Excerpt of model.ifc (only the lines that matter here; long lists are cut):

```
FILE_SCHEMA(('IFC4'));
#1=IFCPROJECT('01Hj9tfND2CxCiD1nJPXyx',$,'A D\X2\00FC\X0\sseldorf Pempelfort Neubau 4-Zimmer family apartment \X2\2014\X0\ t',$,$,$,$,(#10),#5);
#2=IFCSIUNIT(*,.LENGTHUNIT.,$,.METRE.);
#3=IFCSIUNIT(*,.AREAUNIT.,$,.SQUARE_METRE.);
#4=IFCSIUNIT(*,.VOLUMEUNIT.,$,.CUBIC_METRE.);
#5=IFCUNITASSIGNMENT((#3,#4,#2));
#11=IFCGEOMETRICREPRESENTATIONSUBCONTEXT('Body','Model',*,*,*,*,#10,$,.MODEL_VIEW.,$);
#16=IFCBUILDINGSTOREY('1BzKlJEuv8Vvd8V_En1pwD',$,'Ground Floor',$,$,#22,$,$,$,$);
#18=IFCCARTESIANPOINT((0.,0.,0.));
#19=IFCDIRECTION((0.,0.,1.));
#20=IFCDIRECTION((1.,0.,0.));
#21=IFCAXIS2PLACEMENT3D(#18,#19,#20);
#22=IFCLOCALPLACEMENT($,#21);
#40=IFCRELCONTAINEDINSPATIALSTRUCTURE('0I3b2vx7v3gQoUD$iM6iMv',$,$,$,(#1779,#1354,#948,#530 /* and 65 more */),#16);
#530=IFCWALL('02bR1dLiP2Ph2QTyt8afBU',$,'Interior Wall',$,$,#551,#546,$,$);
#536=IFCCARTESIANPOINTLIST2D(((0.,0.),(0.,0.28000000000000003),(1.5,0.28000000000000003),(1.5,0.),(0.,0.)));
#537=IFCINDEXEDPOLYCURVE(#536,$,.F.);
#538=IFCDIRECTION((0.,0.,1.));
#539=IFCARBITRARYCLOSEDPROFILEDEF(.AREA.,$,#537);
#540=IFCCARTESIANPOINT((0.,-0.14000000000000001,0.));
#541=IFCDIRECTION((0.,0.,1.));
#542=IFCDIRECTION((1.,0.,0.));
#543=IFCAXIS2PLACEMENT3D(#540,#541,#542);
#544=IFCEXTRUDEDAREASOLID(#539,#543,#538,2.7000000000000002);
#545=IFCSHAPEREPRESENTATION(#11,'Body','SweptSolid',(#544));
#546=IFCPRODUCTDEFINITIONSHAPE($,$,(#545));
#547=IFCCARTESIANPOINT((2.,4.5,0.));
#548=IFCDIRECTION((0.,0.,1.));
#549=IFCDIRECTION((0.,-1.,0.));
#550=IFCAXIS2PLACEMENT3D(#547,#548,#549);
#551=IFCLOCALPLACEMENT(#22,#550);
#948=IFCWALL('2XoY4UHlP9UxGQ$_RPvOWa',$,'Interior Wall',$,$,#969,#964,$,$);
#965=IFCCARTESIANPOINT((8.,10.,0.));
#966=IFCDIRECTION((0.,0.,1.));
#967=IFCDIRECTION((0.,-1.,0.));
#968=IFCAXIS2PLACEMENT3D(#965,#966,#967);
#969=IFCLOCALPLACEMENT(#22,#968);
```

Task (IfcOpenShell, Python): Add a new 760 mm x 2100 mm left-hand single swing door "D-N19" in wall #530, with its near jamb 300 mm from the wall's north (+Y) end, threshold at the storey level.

```python
import numpy as np
import ifcopenshell
import ifcopenshell.api.feature
import ifcopenshell.api.geometry
import ifcopenshell.api.root
import ifcopenshell.api.spatial
import ifcopenshell.geom
import ifcopenshell.util.element
import ifcopenshell.util.placement
import ifcopenshell.util.representation
import ifcopenshell.util.shape
import ifcopenshell.util.unit

model = ifcopenshell.open("model.ifc")
unit_scale = ifcopenshell.util.unit.calculate_unit_scale(model)
settings = ifcopenshell.geom.settings()


def volume(element):
    """Net volume in cubic metres, openings subtracted."""
    shape = ifcopenshell.geom.create_shape(settings, element)
    return ifcopenshell.util.shape.get_volume(shape.geometry)


wall = model.by_guid("02bR1dLiP2Ph2QTyt8afBU")
storey = ifcopenshell.util.element.get_container(wall, ifc_class="IfcBuildingStorey")
context = ifcopenshell.util.representation.get_context(model, "Model", "Body", "MODEL_VIEW")
before = volume(wall)

width, height, from_end, sill = 0.76, 2.1, 0.3, 0.0  # metres

# The wall runs along its own X axis, and the end named is its -X end.
wall_shape = ifcopenshell.geom.create_shape(settings, wall)
x, y, z = ifcopenshell.util.shape.get_vertices(wall_shape.geometry).T
start = x.min() + from_end
face, thickness = float(y.min()), float(y.max() - y.min())
wall_matrix = ifcopenshell.util.placement.get_local_placement(wall.ObjectPlacement)
level = ifcopenshell.util.placement.get_local_placement(storey.ObjectPlacement)[2, 3]


def in_wall(x, y):
    """Placement at x, y metres in the wall's axes, at sill height."""
    matrix = wall_matrix.copy()
    matrix[:, 3] = wall_matrix @ np.array([x / unit_scale, y / unit_scale, 0.0, 1.0])
    matrix[2, 3] = level + sill / unit_scale
    return matrix


# Opening: a box that overshoots both wall faces by 50 mm.
opening = ifcopenshell.api.root.create_entity(model, ifc_class="IfcOpeningElement", predefined_type="OPENING")
box = ifcopenshell.api.geometry.add_wall_representation(
    model, context=context, length=width, height=height, thickness=thickness + 0.1
)
ifcopenshell.api.geometry.assign_representation(model, product=opening, representation=box)
ifcopenshell.api.geometry.edit_object_placement(model, product=opening, matrix=in_wall(start, face - 0.05), is_si=False)
ifcopenshell.api.feature.add_feature(model, feature=opening, element=wall)

door = ifcopenshell.api.root.create_entity(model, ifc_class="IfcDoor", name="D-N19", predefined_type="DOOR")
door.OverallWidth, door.OverallHeight = width / unit_scale, height / unit_scale
door.OperationType = "SINGLE_SWING_LEFT"
body = ifcopenshell.api.geometry.add_door_representation(
    model,
    context=context,
    overall_width=door.OverallWidth,
    overall_height=door.OverallHeight,
    operation_type="SINGLE_SWING_LEFT",
    lining_properties={"LiningDepth": thickness / unit_scale, "ThresholdDepth": thickness / unit_scale},
)
ifcopenshell.api.geometry.assign_representation(model, product=door, representation=body)
ifcopenshell.api.spatial.assign_container(model, products=[door], relating_structure=storey)
ifcopenshell.api.feature.add_filling(model, opening=opening, element=door)

# The lining spans the wall, so the door starts at the wall face.
ifcopenshell.api.geometry.edit_object_placement(model, product=door, matrix=in_wall(start, face), is_si=False)

after = volume(wall)

print(f"wall volume {before:.3f} -> {after:.3f} m3")

model.write("model-out.ifc")
```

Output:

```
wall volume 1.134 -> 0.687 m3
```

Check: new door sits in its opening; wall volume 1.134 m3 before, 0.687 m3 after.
